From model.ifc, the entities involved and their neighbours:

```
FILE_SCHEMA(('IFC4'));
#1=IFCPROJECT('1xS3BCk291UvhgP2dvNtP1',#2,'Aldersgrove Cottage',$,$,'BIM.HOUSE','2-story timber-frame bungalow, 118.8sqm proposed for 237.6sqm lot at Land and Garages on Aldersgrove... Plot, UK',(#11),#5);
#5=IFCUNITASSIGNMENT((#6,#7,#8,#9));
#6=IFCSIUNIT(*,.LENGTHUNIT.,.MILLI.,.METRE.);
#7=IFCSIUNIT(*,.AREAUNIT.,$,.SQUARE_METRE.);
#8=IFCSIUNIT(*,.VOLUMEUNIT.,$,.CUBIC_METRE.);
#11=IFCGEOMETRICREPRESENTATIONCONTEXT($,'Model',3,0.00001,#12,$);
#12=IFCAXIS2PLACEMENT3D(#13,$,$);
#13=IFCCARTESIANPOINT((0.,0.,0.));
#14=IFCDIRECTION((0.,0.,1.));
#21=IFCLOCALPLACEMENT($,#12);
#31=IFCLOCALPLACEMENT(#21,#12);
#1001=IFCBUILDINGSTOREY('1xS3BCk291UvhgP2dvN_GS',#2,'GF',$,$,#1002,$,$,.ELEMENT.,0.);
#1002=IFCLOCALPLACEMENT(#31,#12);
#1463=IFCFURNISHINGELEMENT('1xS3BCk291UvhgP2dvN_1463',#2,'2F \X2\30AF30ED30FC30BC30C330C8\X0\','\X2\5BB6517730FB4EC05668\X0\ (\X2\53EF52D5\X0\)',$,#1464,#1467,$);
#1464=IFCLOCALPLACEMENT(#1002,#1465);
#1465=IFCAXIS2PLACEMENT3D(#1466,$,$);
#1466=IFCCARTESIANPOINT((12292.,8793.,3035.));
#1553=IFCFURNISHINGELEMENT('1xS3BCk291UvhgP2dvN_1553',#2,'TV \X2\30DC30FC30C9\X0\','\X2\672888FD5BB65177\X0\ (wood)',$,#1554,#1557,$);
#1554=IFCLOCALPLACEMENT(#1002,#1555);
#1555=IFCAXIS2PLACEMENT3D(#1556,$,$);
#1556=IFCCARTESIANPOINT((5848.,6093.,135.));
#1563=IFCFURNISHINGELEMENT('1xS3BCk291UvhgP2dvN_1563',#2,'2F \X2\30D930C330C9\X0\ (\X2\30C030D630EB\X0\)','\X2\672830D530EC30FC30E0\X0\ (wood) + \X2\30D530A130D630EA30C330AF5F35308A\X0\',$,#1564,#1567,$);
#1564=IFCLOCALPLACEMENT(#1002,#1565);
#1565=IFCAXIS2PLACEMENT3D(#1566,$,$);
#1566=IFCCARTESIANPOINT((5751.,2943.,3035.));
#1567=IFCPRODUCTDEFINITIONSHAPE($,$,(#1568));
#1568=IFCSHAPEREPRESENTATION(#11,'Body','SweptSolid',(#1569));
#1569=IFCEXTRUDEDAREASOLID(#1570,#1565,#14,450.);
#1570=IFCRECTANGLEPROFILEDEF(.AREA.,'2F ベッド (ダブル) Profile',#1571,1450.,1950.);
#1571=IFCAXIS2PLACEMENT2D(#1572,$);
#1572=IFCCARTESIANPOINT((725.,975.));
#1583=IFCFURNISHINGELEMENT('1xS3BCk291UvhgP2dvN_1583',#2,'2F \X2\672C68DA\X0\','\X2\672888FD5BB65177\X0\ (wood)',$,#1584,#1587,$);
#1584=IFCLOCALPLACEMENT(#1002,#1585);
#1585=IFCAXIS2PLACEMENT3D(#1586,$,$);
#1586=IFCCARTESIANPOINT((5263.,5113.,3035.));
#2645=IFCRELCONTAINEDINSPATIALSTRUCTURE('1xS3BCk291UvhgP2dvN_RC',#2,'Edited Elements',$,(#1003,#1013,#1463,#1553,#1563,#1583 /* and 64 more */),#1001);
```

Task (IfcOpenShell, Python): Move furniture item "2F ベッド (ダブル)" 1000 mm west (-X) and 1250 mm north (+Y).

```python
import ifcopenshell
import ifcopenshell.api.geometry
import ifcopenshell.util.placement
import ifcopenshell.util.unit

model = ifcopenshell.open("model.ifc")
unit_scale = ifcopenshell.util.unit.calculate_unit_scale(model)

item = model.by_guid("1xS3BCk291UvhgP2dvN_1563")
matrix = ifcopenshell.util.placement.get_local_placement(item.ObjectPlacement)
matrix[0, 3] -= 1 / unit_scale
matrix[1, 3] += 1.25 / unit_scale
ifcopenshell.api.geometry.edit_object_placement(model, product=item, matrix=matrix, is_si=False)

print(ifcopenshell.util.placement.get_local_placement(item.ObjectPlacement).round(3) + 0.0)

model.write("model_edited.ifc")
```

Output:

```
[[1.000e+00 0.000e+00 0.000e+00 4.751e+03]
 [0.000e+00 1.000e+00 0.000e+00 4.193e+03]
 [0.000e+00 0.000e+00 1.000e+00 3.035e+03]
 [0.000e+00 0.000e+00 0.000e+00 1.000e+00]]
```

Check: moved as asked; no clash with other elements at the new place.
